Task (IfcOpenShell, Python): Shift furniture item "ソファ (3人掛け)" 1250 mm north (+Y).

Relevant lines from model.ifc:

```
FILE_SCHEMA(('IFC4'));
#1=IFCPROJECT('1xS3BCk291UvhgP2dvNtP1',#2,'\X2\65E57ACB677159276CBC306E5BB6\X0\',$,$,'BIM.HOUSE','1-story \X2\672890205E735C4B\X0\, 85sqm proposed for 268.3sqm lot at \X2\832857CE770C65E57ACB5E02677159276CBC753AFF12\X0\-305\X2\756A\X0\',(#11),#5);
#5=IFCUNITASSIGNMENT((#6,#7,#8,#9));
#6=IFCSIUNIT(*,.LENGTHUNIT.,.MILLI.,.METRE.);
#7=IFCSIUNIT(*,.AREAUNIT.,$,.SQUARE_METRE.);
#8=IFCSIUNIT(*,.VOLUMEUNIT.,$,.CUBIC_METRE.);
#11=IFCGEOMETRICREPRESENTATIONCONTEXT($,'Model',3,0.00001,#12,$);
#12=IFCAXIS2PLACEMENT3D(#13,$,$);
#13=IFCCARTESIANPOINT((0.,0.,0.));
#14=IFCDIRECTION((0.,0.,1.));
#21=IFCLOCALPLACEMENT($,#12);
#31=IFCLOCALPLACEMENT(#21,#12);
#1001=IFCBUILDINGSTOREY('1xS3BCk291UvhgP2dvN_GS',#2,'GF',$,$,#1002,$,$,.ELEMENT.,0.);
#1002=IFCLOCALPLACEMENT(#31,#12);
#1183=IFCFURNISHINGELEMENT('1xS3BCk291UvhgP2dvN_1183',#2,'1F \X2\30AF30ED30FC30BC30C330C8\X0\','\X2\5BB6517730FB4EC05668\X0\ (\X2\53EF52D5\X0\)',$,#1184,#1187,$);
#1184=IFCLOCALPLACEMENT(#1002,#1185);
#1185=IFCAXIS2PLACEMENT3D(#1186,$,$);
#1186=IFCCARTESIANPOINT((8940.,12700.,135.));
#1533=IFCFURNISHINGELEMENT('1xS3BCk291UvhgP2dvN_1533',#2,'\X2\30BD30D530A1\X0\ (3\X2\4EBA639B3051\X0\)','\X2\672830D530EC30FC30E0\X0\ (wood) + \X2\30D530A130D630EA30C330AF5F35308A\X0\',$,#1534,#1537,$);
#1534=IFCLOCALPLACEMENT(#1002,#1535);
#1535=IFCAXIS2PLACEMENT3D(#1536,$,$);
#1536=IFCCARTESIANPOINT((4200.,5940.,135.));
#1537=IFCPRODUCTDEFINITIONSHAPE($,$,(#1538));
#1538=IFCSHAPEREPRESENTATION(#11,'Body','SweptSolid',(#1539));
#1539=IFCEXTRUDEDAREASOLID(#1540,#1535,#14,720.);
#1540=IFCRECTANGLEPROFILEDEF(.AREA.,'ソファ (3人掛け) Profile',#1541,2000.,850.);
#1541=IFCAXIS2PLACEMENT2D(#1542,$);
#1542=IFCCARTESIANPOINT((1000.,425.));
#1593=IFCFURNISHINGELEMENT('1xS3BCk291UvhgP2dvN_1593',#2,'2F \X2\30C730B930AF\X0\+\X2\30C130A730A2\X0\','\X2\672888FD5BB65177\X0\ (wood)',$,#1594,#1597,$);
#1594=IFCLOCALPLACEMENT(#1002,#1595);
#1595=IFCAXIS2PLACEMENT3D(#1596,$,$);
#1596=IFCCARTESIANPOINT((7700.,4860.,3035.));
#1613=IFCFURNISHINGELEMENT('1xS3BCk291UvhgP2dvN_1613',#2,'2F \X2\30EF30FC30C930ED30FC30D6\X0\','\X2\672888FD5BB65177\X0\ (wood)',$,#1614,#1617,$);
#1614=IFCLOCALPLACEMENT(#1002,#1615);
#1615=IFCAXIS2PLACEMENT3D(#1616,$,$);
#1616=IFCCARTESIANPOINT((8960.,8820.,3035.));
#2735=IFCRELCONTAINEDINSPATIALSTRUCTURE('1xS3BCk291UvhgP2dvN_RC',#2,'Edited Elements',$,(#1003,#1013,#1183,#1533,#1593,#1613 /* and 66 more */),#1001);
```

```python
import ifcopenshell
import ifcopenshell.api.geometry
import ifcopenshell.util.placement
import ifcopenshell.util.unit

model = ifcopenshell.open("model.ifc")
unit_scale = ifcopenshell.util.unit.calculate_unit_scale(model)

item = model.by_guid("1xS3BCk291UvhgP2dvN_1533")
matrix = ifcopenshell.util.placement.get_local_placement(item.ObjectPlacement)
matrix[1, 3] += 1.25 / unit_scale
ifcopenshell.api.geometry.edit_object_placement(model, product=item, matrix=matrix, is_si=False)

print(ifcopenshell.util.placement.get_local_placement(item.ObjectPlacement).round(3) + 0.0)

model.write("model_v2.ifc")
```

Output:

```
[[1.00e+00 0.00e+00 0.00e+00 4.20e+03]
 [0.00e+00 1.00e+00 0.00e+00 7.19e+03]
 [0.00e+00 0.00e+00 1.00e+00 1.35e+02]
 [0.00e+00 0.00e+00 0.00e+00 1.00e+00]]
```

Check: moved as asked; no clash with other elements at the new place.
